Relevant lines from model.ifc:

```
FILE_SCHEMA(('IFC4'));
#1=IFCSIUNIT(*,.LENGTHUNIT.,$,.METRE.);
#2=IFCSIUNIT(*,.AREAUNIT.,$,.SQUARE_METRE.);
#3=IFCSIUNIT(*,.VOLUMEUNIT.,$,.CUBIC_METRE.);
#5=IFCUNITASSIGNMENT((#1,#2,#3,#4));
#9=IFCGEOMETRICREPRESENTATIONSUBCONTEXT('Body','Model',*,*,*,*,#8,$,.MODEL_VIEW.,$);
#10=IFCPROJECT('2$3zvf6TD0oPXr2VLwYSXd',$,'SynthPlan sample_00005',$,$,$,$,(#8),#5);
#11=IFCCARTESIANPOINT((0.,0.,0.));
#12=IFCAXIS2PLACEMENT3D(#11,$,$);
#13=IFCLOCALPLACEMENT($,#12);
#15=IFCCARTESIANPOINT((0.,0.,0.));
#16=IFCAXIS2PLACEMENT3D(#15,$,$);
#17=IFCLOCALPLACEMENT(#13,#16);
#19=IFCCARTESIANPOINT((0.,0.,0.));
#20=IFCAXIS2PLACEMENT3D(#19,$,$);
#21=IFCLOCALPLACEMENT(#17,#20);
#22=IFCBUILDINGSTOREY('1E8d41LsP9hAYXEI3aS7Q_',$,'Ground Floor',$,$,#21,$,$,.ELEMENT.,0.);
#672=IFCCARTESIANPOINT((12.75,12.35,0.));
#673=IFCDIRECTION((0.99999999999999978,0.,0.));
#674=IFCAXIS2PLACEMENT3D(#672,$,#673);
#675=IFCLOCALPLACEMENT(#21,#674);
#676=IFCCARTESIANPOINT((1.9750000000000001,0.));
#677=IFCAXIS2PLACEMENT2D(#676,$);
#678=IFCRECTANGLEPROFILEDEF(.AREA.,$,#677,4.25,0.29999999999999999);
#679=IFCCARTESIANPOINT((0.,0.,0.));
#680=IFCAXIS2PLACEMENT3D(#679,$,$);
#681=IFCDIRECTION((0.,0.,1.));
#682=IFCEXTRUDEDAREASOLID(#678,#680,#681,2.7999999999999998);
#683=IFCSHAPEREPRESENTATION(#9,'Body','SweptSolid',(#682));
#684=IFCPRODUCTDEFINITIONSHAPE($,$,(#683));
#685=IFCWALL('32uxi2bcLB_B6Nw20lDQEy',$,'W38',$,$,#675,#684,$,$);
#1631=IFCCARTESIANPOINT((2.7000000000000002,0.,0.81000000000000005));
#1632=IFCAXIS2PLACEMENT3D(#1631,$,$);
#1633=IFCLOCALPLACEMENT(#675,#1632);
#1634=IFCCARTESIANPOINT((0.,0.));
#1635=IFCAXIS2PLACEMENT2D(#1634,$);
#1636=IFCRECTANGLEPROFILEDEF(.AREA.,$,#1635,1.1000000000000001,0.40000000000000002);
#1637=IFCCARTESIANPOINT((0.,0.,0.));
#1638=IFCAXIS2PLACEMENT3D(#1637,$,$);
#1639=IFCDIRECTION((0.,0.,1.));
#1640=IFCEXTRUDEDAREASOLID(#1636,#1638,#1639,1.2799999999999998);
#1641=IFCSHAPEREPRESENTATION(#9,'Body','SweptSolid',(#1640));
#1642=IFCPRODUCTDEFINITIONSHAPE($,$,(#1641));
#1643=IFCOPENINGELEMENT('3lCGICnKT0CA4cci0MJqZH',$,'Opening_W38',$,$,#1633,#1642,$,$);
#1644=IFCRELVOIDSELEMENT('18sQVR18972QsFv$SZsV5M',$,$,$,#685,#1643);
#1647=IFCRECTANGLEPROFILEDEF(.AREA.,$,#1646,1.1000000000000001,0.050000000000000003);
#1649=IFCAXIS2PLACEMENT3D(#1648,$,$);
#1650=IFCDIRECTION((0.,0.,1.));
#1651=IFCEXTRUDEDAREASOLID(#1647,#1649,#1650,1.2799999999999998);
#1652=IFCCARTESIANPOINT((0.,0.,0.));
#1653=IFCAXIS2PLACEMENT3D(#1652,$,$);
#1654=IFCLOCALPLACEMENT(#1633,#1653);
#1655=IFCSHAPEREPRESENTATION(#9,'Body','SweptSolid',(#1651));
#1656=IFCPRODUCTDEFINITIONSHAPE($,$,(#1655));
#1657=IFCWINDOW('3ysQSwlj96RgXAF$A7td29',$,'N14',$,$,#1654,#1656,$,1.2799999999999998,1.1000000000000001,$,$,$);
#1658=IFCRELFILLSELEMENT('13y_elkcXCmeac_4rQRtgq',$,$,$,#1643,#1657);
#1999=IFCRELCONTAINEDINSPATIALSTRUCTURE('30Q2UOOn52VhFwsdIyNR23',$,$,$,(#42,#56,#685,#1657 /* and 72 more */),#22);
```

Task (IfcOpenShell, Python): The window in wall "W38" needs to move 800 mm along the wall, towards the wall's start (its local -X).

```python
import ifcopenshell
import ifcopenshell.api.geometry
import ifcopenshell.util.placement
import ifcopenshell.util.unit

model = ifcopenshell.open("model.ifc")
unit_scale = ifcopenshell.util.unit.calculate_unit_scale(model)

window = model.by_guid("3ysQSwlj96RgXAF$A7td29")
opening = window.FillsVoids[0].RelatingOpeningElement
wall = opening.VoidsElements[0].RelatingBuildingElement

wall_matrix = ifcopenshell.util.placement.get_local_placement(wall.ObjectPlacement)
shift = wall_matrix[:3, 0] * -0.8 / unit_scale
before = ifcopenshell.util.placement.get_local_placement(window.ObjectPlacement)[:3, 3].copy()

# The window is placed relative to its opening, so it follows when the opening moves.
matrix = ifcopenshell.util.placement.get_local_placement(opening.ObjectPlacement)
matrix[:3, 3] += shift
ifcopenshell.api.geometry.edit_object_placement(
    model, product=opening, matrix=matrix, is_si=False, should_transform_children=True
)

after = ifcopenshell.util.placement.get_local_placement(window.ObjectPlacement)[:3, 3]
print("window moved by", (after - before).round(3) + 0.0)

model.write("model_edited.ifc")
```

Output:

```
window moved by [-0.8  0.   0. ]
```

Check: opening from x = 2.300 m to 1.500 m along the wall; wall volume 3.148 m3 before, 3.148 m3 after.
